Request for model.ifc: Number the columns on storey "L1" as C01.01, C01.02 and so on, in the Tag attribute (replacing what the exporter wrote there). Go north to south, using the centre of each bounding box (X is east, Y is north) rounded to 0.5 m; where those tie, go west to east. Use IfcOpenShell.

First a look at what the model holds.

```python
import ifcopenshell
import ifcopenshell.util.element
import ifcopenshell.util.placement

model = ifcopenshell.open("model.ifc")
print(model.schema)
storey = next(s for s in model.by_type("IfcBuildingStorey") if s.Name == "L1")
columns = [e for e in ifcopenshell.util.element.get_decomposition(storey) if e.is_a("IfcColumn")]
for e in sorted(columns, key=lambda e: e.id()):
    origin = ifcopenshell.util.placement.get_local_placement(e.ObjectPlacement)[:3, 3]
    print(e.id(), e.Tag, e.Name, origin.round(2) + 0.0, sep=" | ")
```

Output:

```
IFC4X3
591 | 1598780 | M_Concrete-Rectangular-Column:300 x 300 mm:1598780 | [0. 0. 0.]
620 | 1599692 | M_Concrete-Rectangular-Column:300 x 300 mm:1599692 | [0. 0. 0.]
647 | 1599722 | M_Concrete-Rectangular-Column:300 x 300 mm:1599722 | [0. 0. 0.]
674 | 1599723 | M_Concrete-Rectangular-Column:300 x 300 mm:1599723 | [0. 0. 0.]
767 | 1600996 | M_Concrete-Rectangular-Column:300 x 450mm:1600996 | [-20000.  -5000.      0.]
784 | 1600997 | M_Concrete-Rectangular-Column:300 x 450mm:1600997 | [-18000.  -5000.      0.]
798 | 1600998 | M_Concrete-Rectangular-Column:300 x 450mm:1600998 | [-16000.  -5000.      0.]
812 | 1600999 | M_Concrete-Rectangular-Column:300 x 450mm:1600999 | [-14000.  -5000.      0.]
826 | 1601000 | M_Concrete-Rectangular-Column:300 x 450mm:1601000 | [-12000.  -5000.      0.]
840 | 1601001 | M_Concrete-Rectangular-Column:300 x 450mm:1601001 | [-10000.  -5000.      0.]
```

```python
import ifcopenshell
import ifcopenshell.geom
import ifcopenshell.util.element
import ifcopenshell.util.shape

model = ifcopenshell.open("model.ifc")
settings = ifcopenshell.geom.settings()
settings.set("use-world-coords", True)


def centre(element):
    shape = ifcopenshell.geom.create_shape(settings, element)
    return ifcopenshell.util.shape.get_bbox_centroid(shape.geometry)


storey = next(s for s in model.by_type("IfcBuildingStorey") if s.Name == "L1")
columns = [e for e in ifcopenshell.util.element.get_decomposition(storey) if e.is_a("IfcColumn")]

# Insertion points can sit at a corner or the storey origin, so sort by the geometry (in metres).
centres = {e: centre(e) for e in columns}
columns.sort(key=lambda e: (-round(centres[e][1] / 0.5), centres[e][0]))

for i, e in enumerate(columns, start=1):
    number = f"C01.{i:02d}"
    e.Tag = number
    print(e.id(), number)

model.write("model_rev.ifc")
```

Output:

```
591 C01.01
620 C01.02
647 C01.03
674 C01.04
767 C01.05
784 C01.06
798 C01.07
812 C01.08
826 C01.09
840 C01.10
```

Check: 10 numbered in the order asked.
